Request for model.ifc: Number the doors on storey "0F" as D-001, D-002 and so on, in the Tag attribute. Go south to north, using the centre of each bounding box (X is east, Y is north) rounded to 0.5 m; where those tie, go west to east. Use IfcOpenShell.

First a look at what the model holds.

```python
import ifcopenshell
import ifcopenshell.util.element
import ifcopenshell.util.placement

model = ifcopenshell.open("model.ifc")
print(model.schema)
storey = next(s for s in model.by_type("IfcBuildingStorey") if s.Name == "0F")
doors = [e for e in ifcopenshell.util.element.get_decomposition(storey) if e.is_a("IfcDoor")]
for e in sorted(doors, key=lambda e: e.id()):
    origin = ifcopenshell.util.placement.get_local_placement(e.ObjectPlacement)[:3, 3]
    print(e.id(), e.Tag, e.Name, origin.round(2) + 0.0, sep=" | ")
```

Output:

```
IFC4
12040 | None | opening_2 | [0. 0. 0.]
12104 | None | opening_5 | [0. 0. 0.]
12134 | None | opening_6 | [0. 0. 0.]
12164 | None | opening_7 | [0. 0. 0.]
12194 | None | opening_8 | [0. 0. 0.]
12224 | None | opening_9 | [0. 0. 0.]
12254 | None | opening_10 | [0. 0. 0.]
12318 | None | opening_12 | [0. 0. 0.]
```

```python
import ifcopenshell
import ifcopenshell.geom
import ifcopenshell.util.element
import ifcopenshell.util.shape

model = ifcopenshell.open("model.ifc")
settings = ifcopenshell.geom.settings()
settings.set("use-world-coords", True)


def centre(element):
    shape = ifcopenshell.geom.create_shape(settings, element)
    return ifcopenshell.util.shape.get_bbox_centroid(shape.geometry)


storey = next(s for s in model.by_type("IfcBuildingStorey") if s.Name == "0F")
doors = [e for e in ifcopenshell.util.element.get_decomposition(storey) if e.is_a("IfcDoor")]

# Insertion points can sit at a corner or the storey origin, so sort by the geometry (in metres).
centres = {e: centre(e) for e in doors}
doors.sort(key=lambda e: (round(centres[e][1] / 0.5), centres[e][0]))

for i, e in enumerate(doors, start=1):
    number = f"D-0{i:02d}"
    e.Tag = number
    print(e.id(), number)

model.write("model_v2.ifc")
```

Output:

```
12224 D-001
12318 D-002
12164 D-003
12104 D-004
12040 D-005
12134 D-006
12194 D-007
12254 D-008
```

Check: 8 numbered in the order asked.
